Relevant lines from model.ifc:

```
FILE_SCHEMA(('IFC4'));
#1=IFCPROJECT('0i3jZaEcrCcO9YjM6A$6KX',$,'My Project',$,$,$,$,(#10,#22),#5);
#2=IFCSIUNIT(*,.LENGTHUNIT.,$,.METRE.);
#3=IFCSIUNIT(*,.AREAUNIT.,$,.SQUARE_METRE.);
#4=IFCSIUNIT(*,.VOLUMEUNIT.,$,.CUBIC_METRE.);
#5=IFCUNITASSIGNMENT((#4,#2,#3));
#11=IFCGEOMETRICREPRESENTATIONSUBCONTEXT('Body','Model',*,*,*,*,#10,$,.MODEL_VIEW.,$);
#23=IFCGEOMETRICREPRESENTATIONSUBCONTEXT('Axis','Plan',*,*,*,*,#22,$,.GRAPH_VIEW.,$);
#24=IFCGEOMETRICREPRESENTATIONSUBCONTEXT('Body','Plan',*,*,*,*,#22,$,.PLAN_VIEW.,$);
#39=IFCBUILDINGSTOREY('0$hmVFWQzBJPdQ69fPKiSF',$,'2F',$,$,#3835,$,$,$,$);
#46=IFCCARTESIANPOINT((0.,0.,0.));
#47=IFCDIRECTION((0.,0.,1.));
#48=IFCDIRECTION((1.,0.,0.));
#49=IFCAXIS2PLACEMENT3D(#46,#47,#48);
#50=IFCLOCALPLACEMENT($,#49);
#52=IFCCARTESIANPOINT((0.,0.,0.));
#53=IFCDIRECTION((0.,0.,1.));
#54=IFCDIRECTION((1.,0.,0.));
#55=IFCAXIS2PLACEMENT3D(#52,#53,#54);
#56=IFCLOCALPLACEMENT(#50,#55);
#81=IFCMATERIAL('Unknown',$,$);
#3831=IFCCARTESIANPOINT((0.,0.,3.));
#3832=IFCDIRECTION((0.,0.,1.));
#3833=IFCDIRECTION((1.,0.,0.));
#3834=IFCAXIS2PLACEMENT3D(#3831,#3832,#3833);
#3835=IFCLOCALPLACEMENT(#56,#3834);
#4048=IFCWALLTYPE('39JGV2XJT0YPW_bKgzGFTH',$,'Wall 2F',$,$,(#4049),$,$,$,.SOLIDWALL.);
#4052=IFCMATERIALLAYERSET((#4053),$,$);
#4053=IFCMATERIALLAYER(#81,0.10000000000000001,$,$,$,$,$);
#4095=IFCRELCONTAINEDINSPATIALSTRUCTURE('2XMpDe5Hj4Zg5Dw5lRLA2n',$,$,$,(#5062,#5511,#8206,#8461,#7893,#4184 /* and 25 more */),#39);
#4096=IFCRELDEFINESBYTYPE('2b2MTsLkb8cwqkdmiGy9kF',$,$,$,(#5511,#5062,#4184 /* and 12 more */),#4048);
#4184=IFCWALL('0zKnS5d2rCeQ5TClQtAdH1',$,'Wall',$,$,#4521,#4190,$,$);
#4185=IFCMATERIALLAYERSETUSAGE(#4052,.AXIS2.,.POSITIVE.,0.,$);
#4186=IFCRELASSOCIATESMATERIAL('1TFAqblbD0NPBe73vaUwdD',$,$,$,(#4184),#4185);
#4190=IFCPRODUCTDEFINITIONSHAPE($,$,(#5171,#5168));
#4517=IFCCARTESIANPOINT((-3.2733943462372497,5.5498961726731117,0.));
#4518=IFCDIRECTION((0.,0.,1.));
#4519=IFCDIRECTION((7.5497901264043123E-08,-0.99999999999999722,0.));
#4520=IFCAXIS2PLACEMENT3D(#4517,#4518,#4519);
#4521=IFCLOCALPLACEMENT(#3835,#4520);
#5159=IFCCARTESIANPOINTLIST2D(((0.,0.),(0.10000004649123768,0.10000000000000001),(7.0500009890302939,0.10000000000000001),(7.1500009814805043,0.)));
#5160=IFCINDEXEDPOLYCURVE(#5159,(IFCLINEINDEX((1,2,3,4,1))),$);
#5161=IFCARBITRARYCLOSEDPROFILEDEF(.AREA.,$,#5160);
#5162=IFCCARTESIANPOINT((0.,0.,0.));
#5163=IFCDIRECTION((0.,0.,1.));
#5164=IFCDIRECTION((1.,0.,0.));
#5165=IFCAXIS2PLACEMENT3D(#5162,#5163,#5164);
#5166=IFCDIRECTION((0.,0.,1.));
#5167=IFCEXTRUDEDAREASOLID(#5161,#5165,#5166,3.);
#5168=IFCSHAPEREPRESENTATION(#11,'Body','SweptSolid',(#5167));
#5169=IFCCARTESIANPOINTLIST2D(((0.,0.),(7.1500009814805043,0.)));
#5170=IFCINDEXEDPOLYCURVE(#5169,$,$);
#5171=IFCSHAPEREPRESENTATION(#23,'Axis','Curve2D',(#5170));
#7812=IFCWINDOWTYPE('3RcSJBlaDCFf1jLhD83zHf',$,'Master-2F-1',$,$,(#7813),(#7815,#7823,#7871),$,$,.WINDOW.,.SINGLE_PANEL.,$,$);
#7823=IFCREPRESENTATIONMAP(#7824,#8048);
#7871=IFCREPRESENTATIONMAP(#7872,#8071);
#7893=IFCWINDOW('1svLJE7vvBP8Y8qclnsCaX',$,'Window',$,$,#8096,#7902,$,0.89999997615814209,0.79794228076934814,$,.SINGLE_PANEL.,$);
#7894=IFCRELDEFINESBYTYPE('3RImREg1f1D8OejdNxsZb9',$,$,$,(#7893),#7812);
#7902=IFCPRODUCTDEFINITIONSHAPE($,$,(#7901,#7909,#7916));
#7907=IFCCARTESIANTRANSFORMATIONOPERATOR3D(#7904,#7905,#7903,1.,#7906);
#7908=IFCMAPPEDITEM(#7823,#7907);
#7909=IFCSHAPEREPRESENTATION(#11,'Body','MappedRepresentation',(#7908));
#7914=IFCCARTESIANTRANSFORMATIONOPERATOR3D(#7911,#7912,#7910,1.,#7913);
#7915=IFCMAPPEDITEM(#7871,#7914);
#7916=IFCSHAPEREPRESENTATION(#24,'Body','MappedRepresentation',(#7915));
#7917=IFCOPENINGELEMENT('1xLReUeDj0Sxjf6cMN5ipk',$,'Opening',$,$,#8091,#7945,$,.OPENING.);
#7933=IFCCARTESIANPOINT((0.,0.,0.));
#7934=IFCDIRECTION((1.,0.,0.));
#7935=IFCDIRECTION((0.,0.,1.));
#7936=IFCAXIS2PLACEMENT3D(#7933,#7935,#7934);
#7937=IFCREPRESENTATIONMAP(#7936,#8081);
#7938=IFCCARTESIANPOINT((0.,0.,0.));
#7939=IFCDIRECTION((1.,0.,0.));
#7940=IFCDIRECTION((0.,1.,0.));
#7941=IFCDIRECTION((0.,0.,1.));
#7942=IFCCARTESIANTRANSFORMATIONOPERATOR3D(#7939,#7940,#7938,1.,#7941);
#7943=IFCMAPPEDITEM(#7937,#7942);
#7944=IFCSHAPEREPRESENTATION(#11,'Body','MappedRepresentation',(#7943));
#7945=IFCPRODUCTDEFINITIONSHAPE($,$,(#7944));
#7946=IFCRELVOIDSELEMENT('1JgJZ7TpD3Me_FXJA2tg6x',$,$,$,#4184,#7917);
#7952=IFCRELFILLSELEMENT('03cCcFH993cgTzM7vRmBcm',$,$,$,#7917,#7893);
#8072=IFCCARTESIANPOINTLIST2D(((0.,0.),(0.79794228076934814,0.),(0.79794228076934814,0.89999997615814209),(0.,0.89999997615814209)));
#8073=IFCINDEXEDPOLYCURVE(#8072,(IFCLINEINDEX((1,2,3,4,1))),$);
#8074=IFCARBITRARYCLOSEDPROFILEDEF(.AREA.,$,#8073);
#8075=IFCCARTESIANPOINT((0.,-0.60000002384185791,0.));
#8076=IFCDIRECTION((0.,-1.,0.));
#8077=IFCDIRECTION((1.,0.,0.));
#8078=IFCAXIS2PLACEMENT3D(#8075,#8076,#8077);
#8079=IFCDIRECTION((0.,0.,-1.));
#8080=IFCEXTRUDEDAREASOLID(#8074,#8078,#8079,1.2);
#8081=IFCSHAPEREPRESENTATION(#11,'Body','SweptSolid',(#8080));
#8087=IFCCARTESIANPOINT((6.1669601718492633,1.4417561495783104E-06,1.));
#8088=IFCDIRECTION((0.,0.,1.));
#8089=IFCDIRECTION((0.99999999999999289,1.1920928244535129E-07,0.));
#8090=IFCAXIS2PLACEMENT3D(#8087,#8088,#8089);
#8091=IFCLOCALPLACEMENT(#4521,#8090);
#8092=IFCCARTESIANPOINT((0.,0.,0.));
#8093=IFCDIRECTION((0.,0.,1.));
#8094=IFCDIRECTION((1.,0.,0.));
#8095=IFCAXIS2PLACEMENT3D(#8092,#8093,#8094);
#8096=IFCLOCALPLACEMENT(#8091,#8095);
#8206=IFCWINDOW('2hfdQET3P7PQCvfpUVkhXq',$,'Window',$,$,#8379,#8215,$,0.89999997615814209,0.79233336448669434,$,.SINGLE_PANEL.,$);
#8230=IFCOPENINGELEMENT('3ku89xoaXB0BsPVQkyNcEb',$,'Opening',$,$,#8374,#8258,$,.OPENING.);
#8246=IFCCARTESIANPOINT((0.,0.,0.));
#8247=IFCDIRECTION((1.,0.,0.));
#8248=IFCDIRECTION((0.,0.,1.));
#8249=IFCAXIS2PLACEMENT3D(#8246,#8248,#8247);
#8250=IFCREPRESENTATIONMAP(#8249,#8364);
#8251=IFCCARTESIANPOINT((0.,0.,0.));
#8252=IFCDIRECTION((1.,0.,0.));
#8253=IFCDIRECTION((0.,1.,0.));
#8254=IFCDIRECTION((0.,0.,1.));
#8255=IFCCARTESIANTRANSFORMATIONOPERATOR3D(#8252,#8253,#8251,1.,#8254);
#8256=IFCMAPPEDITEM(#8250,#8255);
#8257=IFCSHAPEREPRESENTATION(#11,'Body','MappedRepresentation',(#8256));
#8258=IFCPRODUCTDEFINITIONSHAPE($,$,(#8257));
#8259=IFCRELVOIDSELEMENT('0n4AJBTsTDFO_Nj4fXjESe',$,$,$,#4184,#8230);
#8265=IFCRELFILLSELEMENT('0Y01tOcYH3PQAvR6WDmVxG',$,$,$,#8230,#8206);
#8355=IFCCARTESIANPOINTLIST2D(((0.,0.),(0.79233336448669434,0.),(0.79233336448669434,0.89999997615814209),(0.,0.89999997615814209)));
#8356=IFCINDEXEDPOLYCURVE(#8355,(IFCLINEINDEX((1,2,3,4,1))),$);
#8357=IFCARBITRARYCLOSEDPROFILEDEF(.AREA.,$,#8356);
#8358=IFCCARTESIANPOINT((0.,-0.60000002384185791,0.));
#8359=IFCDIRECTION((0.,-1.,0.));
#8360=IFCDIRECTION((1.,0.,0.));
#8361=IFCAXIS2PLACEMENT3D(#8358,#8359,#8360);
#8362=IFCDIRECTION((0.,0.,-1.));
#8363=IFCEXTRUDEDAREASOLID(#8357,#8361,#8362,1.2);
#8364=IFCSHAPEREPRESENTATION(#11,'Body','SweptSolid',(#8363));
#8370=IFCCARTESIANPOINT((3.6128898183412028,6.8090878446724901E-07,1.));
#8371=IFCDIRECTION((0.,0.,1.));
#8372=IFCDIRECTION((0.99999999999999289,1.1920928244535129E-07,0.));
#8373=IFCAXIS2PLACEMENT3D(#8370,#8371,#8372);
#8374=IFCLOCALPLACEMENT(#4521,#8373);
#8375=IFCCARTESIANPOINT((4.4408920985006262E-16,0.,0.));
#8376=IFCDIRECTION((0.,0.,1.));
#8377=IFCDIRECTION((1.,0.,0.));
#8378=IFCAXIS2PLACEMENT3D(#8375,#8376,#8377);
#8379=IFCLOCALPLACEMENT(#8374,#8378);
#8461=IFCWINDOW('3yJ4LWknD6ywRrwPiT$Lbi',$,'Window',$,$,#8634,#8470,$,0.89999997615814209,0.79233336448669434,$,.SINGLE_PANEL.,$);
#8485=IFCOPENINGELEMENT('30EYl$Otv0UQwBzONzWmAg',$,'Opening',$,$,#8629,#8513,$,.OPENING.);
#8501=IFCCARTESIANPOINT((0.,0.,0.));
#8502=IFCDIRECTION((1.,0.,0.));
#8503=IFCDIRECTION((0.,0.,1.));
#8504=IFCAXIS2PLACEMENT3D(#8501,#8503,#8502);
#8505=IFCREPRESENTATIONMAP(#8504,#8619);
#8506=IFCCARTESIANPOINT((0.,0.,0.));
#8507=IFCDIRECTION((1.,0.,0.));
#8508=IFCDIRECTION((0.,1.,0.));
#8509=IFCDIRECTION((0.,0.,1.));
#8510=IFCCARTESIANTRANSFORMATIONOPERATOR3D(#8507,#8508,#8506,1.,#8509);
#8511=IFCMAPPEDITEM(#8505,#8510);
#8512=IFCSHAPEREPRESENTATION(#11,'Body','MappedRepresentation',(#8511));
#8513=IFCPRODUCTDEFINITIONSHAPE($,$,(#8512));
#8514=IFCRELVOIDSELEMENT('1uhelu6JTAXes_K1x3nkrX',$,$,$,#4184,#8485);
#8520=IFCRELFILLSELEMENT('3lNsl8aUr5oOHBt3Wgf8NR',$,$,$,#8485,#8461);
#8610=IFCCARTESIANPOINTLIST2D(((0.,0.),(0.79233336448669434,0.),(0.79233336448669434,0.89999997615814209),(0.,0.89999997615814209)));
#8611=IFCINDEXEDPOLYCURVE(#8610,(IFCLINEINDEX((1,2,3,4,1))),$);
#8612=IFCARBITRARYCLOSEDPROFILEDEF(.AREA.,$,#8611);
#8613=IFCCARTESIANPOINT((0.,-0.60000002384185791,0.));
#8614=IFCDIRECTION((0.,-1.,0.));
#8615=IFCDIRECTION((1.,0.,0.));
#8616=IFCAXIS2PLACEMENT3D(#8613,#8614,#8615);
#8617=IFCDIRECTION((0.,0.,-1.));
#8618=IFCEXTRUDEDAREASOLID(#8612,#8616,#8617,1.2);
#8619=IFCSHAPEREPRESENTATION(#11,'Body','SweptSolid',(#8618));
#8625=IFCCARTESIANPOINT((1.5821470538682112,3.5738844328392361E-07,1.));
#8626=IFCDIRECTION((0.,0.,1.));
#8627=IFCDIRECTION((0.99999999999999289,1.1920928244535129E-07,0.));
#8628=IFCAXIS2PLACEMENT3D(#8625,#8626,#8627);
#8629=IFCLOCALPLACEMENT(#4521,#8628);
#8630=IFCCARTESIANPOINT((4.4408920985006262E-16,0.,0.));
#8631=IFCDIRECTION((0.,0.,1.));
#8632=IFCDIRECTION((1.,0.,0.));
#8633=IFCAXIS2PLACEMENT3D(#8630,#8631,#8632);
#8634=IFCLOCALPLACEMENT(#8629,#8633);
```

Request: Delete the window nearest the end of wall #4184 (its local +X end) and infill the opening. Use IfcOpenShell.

```python
import ifcopenshell
import ifcopenshell.api.feature
import ifcopenshell.api.root
import ifcopenshell.geom
import ifcopenshell.util.shape

model = ifcopenshell.open("model.ifc")
settings = ifcopenshell.geom.settings()


def volume(element):
    """Net volume in cubic metres, openings subtracted."""
    shape = ifcopenshell.geom.create_shape(settings, element)
    return ifcopenshell.util.shape.get_volume(shape.geometry)


window = model.by_guid("1svLJE7vvBP8Y8qclnsCaX")
opening = window.FillsVoids[0].RelatingOpeningElement
wall = opening.VoidsElements[0].RelatingBuildingElement
before = volume(wall)

ifcopenshell.api.root.remove_product(model, product=window)
ifcopenshell.api.feature.remove_feature(model, feature=opening)

after = volume(wall)

print(f"wall volume {before:.3f} -> {after:.3f} m3")

model.write("model-out.ifc")
```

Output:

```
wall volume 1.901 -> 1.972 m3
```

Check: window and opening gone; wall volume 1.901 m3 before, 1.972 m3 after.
